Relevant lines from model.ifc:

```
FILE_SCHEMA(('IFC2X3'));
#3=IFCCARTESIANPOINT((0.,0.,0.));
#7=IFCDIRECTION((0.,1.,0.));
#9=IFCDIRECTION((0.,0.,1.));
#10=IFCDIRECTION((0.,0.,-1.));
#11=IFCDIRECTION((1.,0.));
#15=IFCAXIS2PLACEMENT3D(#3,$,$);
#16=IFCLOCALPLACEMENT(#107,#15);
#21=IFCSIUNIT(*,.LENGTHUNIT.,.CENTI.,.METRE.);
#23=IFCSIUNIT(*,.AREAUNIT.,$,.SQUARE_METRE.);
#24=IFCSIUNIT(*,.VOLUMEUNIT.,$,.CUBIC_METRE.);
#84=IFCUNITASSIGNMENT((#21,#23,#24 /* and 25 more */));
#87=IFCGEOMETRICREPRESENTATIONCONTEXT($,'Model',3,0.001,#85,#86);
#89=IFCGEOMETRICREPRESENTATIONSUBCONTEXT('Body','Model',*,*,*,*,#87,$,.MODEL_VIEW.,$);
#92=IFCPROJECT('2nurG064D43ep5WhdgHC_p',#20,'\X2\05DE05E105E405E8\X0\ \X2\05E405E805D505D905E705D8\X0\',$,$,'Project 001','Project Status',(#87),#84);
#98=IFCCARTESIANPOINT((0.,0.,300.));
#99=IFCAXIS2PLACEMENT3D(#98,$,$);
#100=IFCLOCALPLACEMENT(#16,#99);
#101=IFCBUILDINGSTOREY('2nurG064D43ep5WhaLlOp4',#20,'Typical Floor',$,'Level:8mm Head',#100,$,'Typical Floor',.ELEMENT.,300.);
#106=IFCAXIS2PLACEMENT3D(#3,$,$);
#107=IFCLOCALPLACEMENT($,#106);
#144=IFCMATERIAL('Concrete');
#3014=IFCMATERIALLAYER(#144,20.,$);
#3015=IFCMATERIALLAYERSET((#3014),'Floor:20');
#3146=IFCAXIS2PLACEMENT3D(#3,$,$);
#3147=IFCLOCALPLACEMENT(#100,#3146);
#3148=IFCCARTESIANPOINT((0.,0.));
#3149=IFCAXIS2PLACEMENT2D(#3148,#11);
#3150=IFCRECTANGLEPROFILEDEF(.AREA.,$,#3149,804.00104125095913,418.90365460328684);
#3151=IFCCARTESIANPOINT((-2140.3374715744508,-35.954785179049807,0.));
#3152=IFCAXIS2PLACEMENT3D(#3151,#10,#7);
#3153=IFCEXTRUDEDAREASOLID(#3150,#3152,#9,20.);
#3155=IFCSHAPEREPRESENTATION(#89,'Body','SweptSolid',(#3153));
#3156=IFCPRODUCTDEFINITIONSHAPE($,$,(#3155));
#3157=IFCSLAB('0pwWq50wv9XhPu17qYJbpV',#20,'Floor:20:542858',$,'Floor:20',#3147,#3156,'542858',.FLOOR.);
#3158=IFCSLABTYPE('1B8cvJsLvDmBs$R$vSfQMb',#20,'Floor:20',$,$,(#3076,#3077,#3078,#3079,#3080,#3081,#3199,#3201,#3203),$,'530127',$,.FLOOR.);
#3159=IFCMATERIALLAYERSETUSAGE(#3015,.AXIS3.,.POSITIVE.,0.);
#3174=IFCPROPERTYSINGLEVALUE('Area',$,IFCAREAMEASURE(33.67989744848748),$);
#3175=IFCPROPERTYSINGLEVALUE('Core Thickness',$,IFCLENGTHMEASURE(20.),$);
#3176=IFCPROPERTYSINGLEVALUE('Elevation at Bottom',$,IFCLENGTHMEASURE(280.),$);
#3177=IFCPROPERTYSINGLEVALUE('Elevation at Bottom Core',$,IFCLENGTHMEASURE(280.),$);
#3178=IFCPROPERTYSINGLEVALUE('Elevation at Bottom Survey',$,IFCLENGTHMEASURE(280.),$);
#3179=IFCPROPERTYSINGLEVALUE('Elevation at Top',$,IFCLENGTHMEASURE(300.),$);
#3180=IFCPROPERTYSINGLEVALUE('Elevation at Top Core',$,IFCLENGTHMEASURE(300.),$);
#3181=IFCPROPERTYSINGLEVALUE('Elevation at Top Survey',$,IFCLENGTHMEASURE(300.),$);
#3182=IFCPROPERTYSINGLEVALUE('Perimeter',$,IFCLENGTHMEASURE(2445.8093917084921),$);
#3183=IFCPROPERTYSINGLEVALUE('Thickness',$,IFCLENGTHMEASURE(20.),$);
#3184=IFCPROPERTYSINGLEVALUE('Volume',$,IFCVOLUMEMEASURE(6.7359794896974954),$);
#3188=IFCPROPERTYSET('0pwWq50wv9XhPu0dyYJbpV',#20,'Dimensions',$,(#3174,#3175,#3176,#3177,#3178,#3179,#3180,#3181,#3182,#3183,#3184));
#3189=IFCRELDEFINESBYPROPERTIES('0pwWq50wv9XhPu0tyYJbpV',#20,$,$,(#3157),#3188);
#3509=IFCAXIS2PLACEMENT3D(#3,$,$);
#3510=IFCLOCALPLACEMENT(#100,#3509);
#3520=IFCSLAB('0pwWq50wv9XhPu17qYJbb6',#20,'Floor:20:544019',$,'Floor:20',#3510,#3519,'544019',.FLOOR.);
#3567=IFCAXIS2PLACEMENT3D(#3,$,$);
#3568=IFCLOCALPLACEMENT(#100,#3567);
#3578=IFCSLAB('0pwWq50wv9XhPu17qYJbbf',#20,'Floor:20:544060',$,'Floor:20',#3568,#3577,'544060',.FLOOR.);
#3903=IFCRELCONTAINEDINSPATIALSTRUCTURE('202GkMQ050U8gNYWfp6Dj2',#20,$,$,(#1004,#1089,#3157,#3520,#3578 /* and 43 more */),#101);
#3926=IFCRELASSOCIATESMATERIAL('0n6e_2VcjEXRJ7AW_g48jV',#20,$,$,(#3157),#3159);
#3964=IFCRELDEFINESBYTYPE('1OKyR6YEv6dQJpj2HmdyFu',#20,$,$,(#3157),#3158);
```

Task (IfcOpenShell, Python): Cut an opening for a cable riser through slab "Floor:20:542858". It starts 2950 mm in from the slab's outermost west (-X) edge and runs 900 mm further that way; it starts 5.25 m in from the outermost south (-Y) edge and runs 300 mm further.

```python
import numpy as np
import ifcopenshell
import ifcopenshell.api.feature
import ifcopenshell.api.geometry
import ifcopenshell.api.pset
import ifcopenshell.api.root
import ifcopenshell.geom
import ifcopenshell.util.element
import ifcopenshell.util.placement
import ifcopenshell.util.representation
import ifcopenshell.util.shape
import ifcopenshell.util.unit

model = ifcopenshell.open("model.ifc")
unit_scale = ifcopenshell.util.unit.calculate_unit_scale(model)
area_scale = ifcopenshell.util.unit.calculate_unit_scale(model, "AREAUNIT")
volume_scale = ifcopenshell.util.unit.calculate_unit_scale(model, "VOLUMEUNIT")
settings = ifcopenshell.geom.settings()


def volume(element):
    """Net volume in cubic metres, openings subtracted."""
    shape = ifcopenshell.geom.create_shape(settings, element)
    return ifcopenshell.util.shape.get_volume(shape.geometry)


slab = model.by_id(3157)
before = volume(slab)

# Extent in the slab's own axes, in metres. The edges named are its -X and -Y sides.
slab_shape = ifcopenshell.geom.create_shape(settings, slab)
vertices = ifcopenshell.util.shape.get_vertices(slab_shape.geometry)
x_min, y_min, bottom = vertices.min(axis=0)
top = vertices[:, 2].max()

opening = ifcopenshell.api.root.create_entity(model, ifc_class="IfcOpeningElement", name="Cable riser opening")
context = ifcopenshell.util.representation.get_context(model, "Model", "Body", "MODEL_VIEW")
width, depth = 0.9, 0.3
outline = [(0.0, 0.0), (width, 0.0), (width, depth), (0.0, depth), (0.0, 0.0)]
# Overshoot both faces by 50 mm so the cut is clean.
shape = ifcopenshell.api.geometry.add_slab_representation(
    model, context=context, depth=top - bottom + 0.1, polyline=outline
)
ifcopenshell.api.geometry.assign_representation(model, product=opening, representation=shape)

matrix = ifcopenshell.util.placement.get_local_placement(slab.ObjectPlacement)
matrix[:, 3] = matrix @ np.append(np.array([x_min + 2.95, y_min + 5.25, bottom - 0.05]) / unit_scale, 1.0)
ifcopenshell.api.geometry.edit_object_placement(model, product=opening, matrix=matrix, is_si=False)
ifcopenshell.api.feature.add_feature(model, feature=opening, element=slab)

after = volume(slab)

# Update the slab's stored quantities.
pset = model.by_id(ifcopenshell.util.element.get_pset(slab, "Dimensions", should_inherit=False)["id"])
ifcopenshell.api.pset.edit_pset(model, pset=pset, properties={
    "Area": model.create_entity("IfcAreaMeasure", after / (top - bottom) / area_scale),
    "Volume": model.create_entity("IfcVolumeMeasure", after / volume_scale),
})

print(f"slab volume {before:.3f} -> {after:.3f} m3")

model.write("model_updated.ifc")
```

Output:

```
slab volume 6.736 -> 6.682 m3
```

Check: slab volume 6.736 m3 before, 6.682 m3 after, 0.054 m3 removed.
